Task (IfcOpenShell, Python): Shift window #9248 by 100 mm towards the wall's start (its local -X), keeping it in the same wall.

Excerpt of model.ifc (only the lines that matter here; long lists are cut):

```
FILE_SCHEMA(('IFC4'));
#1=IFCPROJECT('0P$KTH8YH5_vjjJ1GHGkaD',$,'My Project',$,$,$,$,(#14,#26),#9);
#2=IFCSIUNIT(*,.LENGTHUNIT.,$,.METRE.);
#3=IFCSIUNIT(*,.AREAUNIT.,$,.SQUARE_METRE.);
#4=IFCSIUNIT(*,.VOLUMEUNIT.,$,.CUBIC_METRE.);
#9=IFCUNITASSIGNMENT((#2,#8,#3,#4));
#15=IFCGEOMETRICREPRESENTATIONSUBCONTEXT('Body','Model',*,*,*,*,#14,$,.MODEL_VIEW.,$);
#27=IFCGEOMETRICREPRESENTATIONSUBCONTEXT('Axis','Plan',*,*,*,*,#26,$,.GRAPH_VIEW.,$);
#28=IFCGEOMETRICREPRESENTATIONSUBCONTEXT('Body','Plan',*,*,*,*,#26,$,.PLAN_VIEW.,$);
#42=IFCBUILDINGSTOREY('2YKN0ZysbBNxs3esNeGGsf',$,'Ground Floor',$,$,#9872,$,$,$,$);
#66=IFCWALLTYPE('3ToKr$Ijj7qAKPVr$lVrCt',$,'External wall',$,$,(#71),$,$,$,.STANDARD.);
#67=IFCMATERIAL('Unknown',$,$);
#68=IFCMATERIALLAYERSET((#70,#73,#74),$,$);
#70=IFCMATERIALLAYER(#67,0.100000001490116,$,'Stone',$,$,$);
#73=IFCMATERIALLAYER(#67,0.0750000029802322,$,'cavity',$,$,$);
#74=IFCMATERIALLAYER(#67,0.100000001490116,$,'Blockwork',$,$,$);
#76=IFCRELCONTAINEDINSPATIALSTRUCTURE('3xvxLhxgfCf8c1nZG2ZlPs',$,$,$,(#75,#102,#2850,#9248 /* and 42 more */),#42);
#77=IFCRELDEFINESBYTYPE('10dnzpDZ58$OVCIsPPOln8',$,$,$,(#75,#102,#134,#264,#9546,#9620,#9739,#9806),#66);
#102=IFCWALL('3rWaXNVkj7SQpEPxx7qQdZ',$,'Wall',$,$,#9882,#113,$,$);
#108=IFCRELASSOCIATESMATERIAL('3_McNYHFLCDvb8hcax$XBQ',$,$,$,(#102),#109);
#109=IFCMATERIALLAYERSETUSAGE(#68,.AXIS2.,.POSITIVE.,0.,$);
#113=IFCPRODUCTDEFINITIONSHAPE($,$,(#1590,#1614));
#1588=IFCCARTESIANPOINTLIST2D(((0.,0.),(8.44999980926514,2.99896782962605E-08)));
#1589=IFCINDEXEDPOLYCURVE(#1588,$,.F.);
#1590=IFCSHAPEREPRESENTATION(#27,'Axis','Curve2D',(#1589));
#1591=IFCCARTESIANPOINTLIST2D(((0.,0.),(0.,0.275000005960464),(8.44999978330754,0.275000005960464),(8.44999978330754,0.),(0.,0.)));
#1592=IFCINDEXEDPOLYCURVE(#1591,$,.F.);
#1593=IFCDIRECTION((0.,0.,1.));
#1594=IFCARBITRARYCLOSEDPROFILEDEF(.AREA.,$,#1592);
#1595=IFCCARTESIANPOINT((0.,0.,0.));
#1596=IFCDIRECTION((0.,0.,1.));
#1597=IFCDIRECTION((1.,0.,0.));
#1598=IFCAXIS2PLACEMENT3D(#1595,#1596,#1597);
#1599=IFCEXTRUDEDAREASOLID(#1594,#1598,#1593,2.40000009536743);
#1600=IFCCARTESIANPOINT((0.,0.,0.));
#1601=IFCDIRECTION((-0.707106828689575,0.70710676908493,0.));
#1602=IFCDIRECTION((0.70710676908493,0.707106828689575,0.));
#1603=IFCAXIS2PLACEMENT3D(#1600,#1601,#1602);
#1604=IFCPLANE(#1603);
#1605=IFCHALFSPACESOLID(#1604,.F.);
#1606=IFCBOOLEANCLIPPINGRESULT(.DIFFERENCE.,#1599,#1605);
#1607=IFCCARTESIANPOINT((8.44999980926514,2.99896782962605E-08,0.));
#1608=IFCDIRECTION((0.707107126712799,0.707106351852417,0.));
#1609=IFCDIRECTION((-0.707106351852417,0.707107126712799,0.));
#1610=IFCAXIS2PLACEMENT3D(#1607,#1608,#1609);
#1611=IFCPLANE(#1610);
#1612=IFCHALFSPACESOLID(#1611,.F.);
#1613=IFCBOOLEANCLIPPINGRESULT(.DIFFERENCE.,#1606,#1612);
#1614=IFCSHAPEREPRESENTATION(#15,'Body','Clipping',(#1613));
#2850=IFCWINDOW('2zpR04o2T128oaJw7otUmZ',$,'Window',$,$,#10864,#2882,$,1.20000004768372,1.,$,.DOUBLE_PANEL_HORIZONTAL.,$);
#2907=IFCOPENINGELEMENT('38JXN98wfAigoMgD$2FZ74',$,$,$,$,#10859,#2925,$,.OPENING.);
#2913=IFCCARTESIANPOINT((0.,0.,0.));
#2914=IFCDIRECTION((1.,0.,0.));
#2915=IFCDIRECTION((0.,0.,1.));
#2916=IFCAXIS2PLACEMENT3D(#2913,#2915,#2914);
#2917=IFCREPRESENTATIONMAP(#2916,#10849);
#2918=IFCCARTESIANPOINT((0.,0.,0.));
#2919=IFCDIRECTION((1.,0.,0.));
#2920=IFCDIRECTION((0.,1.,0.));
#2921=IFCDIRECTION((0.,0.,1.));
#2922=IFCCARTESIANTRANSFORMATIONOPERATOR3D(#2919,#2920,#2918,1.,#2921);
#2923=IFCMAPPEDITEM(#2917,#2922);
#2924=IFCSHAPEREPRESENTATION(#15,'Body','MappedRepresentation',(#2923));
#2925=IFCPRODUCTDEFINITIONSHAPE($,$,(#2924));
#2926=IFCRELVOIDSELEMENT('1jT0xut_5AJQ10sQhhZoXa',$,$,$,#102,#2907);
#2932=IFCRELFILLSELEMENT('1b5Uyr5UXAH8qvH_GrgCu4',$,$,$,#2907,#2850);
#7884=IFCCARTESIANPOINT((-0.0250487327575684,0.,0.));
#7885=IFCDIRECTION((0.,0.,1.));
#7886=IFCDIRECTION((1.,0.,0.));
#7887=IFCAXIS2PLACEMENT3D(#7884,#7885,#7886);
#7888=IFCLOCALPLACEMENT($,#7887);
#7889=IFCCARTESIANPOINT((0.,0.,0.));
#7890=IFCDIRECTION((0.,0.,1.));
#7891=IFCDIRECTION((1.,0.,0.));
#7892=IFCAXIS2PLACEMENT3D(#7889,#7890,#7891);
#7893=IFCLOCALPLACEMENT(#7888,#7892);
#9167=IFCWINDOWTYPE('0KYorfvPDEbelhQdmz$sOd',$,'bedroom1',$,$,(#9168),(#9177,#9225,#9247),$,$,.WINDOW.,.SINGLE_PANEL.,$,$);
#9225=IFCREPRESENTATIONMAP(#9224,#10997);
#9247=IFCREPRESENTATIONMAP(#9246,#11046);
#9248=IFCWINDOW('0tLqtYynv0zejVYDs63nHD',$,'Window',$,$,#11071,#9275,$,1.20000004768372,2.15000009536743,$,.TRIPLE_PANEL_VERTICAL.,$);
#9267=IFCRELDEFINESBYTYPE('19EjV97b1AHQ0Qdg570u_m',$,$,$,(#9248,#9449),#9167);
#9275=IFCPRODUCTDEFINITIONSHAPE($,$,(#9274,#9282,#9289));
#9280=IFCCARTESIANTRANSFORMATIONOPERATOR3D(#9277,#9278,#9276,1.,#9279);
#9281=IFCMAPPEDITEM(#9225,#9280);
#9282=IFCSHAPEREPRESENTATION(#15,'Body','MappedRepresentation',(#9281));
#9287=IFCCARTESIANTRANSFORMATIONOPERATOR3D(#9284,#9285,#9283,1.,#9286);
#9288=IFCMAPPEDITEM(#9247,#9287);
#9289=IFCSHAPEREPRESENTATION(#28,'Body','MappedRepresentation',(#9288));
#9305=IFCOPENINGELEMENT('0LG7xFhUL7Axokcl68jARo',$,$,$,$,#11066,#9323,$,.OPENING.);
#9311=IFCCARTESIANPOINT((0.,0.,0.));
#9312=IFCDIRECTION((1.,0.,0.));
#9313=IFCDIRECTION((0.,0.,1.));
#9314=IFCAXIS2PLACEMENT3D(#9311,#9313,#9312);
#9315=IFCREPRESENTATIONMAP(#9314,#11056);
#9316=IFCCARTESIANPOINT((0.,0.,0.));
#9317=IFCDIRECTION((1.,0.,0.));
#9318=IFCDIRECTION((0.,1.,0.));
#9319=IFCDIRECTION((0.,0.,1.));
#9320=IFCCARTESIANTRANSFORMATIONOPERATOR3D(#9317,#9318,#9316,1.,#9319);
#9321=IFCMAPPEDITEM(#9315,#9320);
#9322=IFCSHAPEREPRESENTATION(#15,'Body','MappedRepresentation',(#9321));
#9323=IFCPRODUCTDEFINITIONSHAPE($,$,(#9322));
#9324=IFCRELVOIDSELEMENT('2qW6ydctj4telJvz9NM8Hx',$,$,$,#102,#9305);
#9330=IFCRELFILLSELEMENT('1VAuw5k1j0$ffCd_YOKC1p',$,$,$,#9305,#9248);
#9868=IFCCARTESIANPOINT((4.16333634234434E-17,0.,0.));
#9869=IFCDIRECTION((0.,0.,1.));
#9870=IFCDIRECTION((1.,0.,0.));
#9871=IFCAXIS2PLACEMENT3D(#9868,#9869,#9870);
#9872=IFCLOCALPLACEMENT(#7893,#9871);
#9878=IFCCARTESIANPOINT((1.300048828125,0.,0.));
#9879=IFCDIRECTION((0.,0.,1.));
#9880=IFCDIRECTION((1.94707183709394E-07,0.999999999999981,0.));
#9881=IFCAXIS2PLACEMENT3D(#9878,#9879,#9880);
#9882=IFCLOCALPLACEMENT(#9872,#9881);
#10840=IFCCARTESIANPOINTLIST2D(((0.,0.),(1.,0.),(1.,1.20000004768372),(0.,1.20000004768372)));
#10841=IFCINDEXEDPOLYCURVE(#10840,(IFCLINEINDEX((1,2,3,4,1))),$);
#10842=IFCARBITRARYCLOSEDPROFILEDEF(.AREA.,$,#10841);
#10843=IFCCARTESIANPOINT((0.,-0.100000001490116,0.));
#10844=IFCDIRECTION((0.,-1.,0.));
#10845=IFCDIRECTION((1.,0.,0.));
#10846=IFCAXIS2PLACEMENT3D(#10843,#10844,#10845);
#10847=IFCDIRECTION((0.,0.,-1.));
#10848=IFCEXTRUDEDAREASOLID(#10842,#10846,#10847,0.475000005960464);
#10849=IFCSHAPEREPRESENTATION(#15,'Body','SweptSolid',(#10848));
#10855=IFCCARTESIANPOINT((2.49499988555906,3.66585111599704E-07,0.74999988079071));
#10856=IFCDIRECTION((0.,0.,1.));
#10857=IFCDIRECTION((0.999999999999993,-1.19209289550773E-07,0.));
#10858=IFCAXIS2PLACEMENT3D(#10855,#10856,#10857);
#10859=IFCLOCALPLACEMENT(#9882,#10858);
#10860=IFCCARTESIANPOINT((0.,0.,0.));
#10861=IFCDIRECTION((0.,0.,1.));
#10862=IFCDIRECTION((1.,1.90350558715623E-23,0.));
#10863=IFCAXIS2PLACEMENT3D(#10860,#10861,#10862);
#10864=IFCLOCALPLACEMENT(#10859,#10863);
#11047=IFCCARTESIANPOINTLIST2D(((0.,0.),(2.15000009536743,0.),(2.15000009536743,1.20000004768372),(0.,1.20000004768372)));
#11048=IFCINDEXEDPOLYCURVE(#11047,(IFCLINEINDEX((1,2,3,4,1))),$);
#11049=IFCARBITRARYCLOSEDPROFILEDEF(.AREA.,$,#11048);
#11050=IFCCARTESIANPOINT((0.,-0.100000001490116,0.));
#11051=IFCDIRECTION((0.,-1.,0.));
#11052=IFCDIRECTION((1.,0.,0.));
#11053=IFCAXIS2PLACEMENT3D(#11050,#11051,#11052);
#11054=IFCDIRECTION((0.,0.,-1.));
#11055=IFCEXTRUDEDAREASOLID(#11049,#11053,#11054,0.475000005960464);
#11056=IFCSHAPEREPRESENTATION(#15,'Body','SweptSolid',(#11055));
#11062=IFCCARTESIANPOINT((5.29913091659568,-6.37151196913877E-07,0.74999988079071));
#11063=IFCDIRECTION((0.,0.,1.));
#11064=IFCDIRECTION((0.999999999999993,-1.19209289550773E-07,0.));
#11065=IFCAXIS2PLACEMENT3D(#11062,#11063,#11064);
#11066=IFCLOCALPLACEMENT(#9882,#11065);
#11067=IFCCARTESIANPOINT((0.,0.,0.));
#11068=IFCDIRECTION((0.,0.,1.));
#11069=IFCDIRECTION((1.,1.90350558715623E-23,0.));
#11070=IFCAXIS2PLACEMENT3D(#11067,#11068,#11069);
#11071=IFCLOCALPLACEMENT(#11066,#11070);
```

```python
import ifcopenshell
import ifcopenshell.api.geometry
import ifcopenshell.util.placement

model = ifcopenshell.open("model.ifc")

window = model.by_id(9248)
opening = window.FillsVoids[0].RelatingOpeningElement
wall = opening.VoidsElements[0].RelatingBuildingElement

wall_matrix = ifcopenshell.util.placement.get_local_placement(wall.ObjectPlacement)
shift = wall_matrix[:3, 0] * -0.1
before = ifcopenshell.util.placement.get_local_placement(window.ObjectPlacement)[:3, 3].copy()

# The window is placed relative to its opening, so it follows when the opening moves.
matrix = ifcopenshell.util.placement.get_local_placement(opening.ObjectPlacement)
matrix[:3, 3] += shift
ifcopenshell.api.geometry.edit_object_placement(
    model, product=opening, matrix=matrix, is_si=False, should_transform_children=True
)

after = ifcopenshell.util.placement.get_local_placement(window.ObjectPlacement)[:3, 3]
print("window moved by", (after - before).round(3) + 0.0)

model.write("model_updated.ifc")
```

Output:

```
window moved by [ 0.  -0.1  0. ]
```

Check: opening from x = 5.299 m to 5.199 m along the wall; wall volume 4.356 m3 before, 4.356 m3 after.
